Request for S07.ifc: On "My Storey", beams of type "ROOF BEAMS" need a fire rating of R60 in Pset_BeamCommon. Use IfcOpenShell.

First a look at what the model holds.

```python
import ifcopenshell
import ifcopenshell.util.element

model = ifcopenshell.open("S07.ifc")
print(model.schema)
storey = next(s for s in model.by_type("IfcBuildingStorey") if s.Name == "My Storey")
beams = [e for e in ifcopenshell.util.element.get_decomposition(storey) if e.is_a("IfcBeam")]
seen = {}
for e in beams:
    element_type = ifcopenshell.util.element.get_type(e)
    key = (element_type.Name if element_type != e and element_type else None, ifcopenshell.util.element.get_pset(e, "Pset_BeamCommon", "FireRating"))
    seen[key] = seen.get(key, 0) + 1
for (name, value), count in sorted(seen.items(), key=str):
    print(count, "x", name, "|", value)
```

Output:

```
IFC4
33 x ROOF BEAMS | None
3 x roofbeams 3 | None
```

```python
import ifcopenshell
import ifcopenshell.api.pset
import ifcopenshell.util.element

model = ifcopenshell.open("S07.ifc")

storey = next(s for s in model.by_type("IfcBuildingStorey") if s.Name == "My Storey")
beams = [e for e in ifcopenshell.util.element.get_decomposition(storey) if e.is_a("IfcBeam")]

count = 0
for e in beams:
    element_type = ifcopenshell.util.element.get_type(e)
    if element_type in (None, e) or element_type.Name != "ROOF BEAMS":
        continue
    # add_pset returns the element's existing set when there is one.
    pset = ifcopenshell.api.pset.add_pset(model, product=e, name="Pset_BeamCommon")
    ifcopenshell.api.pset.edit_pset(model, pset=pset, properties={"FireRating": "R60"})
    count += 1

print(count, "beams updated")

model.write("S07_rev.ifc")
```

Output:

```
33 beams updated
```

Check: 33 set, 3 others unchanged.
